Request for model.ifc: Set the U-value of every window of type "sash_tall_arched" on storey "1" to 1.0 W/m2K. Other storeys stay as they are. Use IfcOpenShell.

First a look at what the model holds.

```python
import ifcopenshell
import ifcopenshell.util.element

model = ifcopenshell.open("model.ifc")
print(model.schema)
storey = next(s for s in model.by_type("IfcBuildingStorey") if s.Name == "1")
windows = [e for e in ifcopenshell.util.element.get_decomposition(storey) if e.is_a("IfcWindow")]
seen = {}
for e in windows:
    element_type = ifcopenshell.util.element.get_type(e)
    key = (element_type.Name if element_type != e and element_type else None, ifcopenshell.util.element.get_pset(e, "Pset_WindowCommon", "ThermalTransmittance"))
    seen[key] = seen.get(key, 0) + 1
for (name, value), count in sorted(seen.items(), key=str):
    print(count, "x", name, "|", value)
```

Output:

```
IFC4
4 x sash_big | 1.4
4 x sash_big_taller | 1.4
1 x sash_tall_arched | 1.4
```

```python
import ifcopenshell
import ifcopenshell.api.pset
import ifcopenshell.util.element

model = ifcopenshell.open("model.ifc")

storey = next(s for s in model.by_type("IfcBuildingStorey") if s.Name == "1")
windows = [e for e in ifcopenshell.util.element.get_decomposition(storey) if e.is_a("IfcWindow")]

count = 0
for e in windows:
    element_type = ifcopenshell.util.element.get_type(e)
    if element_type in (None, e) or element_type.Name != "sash_tall_arched":
        continue
    # add_pset returns the element's existing set when there is one.
    pset = ifcopenshell.api.pset.add_pset(model, product=e, name="Pset_WindowCommon")
    ifcopenshell.api.pset.edit_pset(model, pset=pset, properties={"ThermalTransmittance": 1.0})
    count += 1

print(count, "windows updated")

model.write("model-out.ifc")
```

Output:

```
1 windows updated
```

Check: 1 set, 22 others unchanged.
